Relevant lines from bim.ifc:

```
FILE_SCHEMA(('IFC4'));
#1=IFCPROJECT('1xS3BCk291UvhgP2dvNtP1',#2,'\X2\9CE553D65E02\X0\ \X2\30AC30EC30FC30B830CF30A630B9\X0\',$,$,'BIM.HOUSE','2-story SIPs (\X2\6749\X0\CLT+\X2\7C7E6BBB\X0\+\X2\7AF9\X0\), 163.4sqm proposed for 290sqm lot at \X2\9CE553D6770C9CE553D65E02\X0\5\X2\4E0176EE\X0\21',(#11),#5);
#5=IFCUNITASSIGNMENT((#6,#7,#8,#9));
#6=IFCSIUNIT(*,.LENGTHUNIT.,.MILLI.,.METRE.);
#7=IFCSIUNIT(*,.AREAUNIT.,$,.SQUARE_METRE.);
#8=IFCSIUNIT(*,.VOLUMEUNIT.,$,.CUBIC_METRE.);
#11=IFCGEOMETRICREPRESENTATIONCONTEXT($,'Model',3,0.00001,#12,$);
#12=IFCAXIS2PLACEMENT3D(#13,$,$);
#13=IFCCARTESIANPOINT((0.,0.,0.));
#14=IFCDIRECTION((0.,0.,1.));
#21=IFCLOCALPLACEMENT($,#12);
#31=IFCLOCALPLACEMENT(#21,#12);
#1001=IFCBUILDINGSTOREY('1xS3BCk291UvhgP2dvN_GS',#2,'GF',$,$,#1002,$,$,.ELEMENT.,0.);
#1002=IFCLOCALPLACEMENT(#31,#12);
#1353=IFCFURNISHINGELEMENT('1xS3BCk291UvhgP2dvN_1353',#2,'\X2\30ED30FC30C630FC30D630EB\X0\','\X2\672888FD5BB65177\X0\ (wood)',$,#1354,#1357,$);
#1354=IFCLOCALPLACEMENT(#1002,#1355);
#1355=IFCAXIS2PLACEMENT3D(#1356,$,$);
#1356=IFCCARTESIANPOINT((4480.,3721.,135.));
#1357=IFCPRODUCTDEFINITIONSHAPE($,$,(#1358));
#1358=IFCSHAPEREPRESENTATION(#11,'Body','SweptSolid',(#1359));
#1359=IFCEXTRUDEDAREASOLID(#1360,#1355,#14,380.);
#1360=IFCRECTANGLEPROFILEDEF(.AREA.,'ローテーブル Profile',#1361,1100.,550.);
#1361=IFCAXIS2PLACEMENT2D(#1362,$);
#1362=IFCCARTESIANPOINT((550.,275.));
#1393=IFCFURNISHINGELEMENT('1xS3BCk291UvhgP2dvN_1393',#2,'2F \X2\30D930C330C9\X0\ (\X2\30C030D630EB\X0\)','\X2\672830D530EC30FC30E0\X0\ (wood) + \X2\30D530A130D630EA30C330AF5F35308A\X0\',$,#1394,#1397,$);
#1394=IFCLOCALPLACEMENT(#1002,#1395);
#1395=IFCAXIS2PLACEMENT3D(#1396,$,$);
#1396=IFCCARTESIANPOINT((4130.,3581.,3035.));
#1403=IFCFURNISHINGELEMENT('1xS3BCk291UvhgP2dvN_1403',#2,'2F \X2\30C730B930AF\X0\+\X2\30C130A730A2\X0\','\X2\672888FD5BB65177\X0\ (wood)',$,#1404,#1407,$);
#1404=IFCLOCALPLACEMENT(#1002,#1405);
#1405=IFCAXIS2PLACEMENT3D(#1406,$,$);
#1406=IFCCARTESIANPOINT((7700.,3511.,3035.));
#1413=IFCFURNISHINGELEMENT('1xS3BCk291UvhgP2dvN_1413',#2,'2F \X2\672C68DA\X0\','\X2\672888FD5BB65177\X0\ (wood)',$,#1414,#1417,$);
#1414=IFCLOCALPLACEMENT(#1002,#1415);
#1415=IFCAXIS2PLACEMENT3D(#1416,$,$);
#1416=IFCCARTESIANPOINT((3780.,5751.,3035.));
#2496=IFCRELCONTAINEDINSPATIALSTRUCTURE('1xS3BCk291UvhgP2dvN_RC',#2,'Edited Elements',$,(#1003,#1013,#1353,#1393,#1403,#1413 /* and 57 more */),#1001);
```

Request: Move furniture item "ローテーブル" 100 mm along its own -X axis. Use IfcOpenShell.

```python
import ifcopenshell
import ifcopenshell.api.geometry
import ifcopenshell.util.placement

model = ifcopenshell.open("bim.ifc")

item = model.by_guid("1xS3BCk291UvhgP2dvN_1353")
matrix = ifcopenshell.util.placement.get_local_placement(item.ObjectPlacement)
matrix[:3, 3] -= matrix[:3, 0] * 100.0
ifcopenshell.api.geometry.edit_object_placement(model, product=item, matrix=matrix, is_si=False)

print(ifcopenshell.util.placement.get_local_placement(item.ObjectPlacement).round(3) + 0.0)

model.write("bim_v2.ifc")
```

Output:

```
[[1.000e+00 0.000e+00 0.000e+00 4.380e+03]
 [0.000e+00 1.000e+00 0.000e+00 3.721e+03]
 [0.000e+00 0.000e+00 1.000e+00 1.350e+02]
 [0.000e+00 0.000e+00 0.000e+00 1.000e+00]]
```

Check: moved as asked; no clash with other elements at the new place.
